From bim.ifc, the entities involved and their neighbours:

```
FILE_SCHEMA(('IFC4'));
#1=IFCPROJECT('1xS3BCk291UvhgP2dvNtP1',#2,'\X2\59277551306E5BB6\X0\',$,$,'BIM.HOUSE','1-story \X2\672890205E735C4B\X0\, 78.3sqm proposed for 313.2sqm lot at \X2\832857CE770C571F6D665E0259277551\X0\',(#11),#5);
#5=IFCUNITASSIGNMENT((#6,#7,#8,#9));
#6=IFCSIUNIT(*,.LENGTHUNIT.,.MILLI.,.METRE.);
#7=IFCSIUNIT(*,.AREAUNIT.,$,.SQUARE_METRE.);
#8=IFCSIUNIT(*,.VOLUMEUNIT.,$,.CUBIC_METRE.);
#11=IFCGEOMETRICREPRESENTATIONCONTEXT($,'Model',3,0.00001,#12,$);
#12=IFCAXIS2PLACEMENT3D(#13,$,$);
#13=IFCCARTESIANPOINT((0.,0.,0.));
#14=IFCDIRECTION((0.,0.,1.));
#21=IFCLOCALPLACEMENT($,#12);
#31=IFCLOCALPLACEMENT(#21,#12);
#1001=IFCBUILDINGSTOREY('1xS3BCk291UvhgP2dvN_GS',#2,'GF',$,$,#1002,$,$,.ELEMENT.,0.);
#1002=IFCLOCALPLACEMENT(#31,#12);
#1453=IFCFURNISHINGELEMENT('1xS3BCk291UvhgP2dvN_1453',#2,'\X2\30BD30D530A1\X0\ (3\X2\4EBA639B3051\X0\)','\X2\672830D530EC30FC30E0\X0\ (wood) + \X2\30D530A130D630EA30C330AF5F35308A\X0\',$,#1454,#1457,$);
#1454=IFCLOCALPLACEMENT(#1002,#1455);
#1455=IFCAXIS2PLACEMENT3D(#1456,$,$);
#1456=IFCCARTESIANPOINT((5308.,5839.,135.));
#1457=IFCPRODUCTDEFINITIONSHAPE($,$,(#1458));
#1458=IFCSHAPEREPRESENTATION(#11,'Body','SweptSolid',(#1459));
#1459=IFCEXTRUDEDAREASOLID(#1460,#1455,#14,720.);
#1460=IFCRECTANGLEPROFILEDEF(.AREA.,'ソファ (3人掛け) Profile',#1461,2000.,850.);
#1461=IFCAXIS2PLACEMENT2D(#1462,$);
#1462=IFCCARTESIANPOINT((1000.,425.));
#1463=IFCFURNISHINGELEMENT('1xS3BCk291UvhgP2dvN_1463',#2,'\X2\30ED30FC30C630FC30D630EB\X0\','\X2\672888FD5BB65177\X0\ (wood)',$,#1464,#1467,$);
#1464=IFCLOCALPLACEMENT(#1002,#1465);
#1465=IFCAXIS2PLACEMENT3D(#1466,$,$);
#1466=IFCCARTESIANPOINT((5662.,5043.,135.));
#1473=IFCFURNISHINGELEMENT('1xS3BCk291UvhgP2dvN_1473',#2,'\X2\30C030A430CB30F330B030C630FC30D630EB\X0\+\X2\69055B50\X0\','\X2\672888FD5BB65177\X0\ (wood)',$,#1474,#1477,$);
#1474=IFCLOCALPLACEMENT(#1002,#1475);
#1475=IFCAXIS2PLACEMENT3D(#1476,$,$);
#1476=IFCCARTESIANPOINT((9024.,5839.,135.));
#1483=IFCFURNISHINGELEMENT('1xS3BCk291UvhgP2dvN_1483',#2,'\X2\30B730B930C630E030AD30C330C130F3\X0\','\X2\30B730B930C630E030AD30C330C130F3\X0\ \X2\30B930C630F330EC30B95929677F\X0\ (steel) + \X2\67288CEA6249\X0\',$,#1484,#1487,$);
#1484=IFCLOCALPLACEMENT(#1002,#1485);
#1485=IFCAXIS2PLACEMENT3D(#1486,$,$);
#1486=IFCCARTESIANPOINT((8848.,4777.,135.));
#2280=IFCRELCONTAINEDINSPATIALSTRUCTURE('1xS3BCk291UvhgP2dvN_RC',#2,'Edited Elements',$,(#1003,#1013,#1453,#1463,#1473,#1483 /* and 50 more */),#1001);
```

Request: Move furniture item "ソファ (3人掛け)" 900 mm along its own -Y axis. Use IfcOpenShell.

```python
import ifcopenshell
import ifcopenshell.api.geometry
import ifcopenshell.util.placement
import ifcopenshell.util.unit

model = ifcopenshell.open("bim.ifc")
unit_scale = ifcopenshell.util.unit.calculate_unit_scale(model)

item = model.by_id(1453)
matrix = ifcopenshell.util.placement.get_local_placement(item.ObjectPlacement)
matrix[:3, 3] -= matrix[:3, 1] * 0.9 / unit_scale
ifcopenshell.api.geometry.edit_object_placement(model, product=item, matrix=matrix, is_si=False)

print(ifcopenshell.util.placement.get_local_placement(item.ObjectPlacement).round(3) + 0.0)

model.write("bim-out.ifc")
```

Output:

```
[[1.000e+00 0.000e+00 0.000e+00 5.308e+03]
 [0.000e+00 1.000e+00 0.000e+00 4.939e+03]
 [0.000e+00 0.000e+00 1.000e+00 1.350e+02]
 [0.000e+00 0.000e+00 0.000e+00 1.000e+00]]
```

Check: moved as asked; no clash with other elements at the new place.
